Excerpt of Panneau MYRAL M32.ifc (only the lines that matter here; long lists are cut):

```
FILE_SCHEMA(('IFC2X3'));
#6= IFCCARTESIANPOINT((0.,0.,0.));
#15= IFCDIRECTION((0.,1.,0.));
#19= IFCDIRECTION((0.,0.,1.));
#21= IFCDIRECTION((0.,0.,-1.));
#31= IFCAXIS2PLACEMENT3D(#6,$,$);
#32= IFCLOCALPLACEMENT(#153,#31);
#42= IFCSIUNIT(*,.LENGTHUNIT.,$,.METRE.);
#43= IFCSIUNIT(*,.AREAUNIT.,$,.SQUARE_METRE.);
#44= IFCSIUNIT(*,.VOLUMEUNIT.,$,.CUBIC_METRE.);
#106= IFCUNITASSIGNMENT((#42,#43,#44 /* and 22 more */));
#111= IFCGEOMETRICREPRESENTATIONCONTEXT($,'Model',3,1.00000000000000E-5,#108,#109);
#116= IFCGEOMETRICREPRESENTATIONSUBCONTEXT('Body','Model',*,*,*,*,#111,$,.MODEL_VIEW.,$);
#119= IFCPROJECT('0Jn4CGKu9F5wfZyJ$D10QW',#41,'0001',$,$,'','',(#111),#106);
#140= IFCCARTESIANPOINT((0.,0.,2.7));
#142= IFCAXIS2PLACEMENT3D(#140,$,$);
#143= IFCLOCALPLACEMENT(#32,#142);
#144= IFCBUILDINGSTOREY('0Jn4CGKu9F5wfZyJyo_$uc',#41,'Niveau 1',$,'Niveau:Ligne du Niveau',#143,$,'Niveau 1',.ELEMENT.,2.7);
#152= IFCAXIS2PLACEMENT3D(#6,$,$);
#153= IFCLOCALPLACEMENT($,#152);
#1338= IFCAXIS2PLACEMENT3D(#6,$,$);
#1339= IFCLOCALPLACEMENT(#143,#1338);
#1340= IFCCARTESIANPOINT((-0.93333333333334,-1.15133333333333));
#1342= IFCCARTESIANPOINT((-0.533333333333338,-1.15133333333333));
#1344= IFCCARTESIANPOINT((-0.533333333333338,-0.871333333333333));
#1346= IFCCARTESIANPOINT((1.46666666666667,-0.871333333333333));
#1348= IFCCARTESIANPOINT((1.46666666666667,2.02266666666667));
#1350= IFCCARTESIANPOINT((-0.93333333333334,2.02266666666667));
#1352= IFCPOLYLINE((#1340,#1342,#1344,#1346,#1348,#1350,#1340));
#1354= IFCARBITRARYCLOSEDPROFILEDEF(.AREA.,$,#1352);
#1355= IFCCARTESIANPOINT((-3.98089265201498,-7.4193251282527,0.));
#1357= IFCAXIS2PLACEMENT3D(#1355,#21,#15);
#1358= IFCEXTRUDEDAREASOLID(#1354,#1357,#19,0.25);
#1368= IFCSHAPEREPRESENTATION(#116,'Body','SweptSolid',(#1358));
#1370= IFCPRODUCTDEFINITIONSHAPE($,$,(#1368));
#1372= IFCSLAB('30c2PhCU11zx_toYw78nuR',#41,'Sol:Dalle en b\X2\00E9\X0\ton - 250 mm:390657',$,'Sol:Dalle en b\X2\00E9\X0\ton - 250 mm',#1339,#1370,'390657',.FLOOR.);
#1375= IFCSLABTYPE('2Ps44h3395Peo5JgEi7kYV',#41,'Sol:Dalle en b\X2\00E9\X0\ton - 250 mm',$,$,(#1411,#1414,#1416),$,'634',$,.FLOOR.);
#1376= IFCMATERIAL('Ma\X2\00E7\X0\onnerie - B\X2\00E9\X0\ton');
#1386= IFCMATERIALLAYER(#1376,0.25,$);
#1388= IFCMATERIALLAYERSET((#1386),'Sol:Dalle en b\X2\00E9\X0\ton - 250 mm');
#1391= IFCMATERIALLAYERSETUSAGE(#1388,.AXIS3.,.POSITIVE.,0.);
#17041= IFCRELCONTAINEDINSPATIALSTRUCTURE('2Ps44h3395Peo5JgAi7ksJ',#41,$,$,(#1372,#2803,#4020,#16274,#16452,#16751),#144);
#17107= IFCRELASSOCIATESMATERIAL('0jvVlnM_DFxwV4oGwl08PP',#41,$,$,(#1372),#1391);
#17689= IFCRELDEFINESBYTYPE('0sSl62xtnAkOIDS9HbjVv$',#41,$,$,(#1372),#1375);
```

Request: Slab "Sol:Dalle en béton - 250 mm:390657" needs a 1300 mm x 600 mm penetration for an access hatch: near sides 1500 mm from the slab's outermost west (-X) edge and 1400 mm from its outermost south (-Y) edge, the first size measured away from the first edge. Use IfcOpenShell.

```python
import numpy as np
import ifcopenshell
import ifcopenshell.api.feature
import ifcopenshell.api.geometry
import ifcopenshell.api.root
import ifcopenshell.geom
import ifcopenshell.util.placement
import ifcopenshell.util.representation
import ifcopenshell.util.shape
import ifcopenshell.util.unit

model = ifcopenshell.open("Panneau MYRAL M32.ifc")
unit_scale = ifcopenshell.util.unit.calculate_unit_scale(model)
settings = ifcopenshell.geom.settings()


def volume(element):
    """Net volume in cubic metres, openings subtracted."""
    shape = ifcopenshell.geom.create_shape(settings, element)
    return ifcopenshell.util.shape.get_volume(shape.geometry)


slab = model.by_guid("30c2PhCU11zx_toYw78nuR")
before = volume(slab)

# Extent in the slab's own axes, in metres. The edges named are its -X and -Y sides.
slab_shape = ifcopenshell.geom.create_shape(settings, slab)
vertices = ifcopenshell.util.shape.get_vertices(slab_shape.geometry)
x_min, y_min, bottom = vertices.min(axis=0)
top = vertices[:, 2].max()

opening = ifcopenshell.api.root.create_entity(model, ifc_class="IfcOpeningElement", name="Access hatch opening")
context = ifcopenshell.util.representation.get_context(model, "Model", "Body", "MODEL_VIEW")
width, depth = 1.3, 0.6
outline = [(0.0, 0.0), (width, 0.0), (width, depth), (0.0, depth), (0.0, 0.0)]
# Overshoot both faces by 50 mm so the cut is clean.
shape = ifcopenshell.api.geometry.add_slab_representation(
    model, context=context, depth=top - bottom + 0.1, polyline=outline
)
ifcopenshell.api.geometry.assign_representation(model, product=opening, representation=shape)

matrix = ifcopenshell.util.placement.get_local_placement(slab.ObjectPlacement)
matrix[:, 3] = matrix @ np.append(np.array([x_min + 1.5, y_min + 1.4, bottom - 0.05]) / unit_scale, 1.0)
ifcopenshell.api.geometry.edit_object_placement(model, product=opening, matrix=matrix, is_si=False)
ifcopenshell.api.feature.add_feature(model, feature=opening, element=slab)

after = volume(slab)

print(f"slab volume {before:.3f} -> {after:.3f} m3")

model.write("Panneau MYRAL M32_edited.ifc")
```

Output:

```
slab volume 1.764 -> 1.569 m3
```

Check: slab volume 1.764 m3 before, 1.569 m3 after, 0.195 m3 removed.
